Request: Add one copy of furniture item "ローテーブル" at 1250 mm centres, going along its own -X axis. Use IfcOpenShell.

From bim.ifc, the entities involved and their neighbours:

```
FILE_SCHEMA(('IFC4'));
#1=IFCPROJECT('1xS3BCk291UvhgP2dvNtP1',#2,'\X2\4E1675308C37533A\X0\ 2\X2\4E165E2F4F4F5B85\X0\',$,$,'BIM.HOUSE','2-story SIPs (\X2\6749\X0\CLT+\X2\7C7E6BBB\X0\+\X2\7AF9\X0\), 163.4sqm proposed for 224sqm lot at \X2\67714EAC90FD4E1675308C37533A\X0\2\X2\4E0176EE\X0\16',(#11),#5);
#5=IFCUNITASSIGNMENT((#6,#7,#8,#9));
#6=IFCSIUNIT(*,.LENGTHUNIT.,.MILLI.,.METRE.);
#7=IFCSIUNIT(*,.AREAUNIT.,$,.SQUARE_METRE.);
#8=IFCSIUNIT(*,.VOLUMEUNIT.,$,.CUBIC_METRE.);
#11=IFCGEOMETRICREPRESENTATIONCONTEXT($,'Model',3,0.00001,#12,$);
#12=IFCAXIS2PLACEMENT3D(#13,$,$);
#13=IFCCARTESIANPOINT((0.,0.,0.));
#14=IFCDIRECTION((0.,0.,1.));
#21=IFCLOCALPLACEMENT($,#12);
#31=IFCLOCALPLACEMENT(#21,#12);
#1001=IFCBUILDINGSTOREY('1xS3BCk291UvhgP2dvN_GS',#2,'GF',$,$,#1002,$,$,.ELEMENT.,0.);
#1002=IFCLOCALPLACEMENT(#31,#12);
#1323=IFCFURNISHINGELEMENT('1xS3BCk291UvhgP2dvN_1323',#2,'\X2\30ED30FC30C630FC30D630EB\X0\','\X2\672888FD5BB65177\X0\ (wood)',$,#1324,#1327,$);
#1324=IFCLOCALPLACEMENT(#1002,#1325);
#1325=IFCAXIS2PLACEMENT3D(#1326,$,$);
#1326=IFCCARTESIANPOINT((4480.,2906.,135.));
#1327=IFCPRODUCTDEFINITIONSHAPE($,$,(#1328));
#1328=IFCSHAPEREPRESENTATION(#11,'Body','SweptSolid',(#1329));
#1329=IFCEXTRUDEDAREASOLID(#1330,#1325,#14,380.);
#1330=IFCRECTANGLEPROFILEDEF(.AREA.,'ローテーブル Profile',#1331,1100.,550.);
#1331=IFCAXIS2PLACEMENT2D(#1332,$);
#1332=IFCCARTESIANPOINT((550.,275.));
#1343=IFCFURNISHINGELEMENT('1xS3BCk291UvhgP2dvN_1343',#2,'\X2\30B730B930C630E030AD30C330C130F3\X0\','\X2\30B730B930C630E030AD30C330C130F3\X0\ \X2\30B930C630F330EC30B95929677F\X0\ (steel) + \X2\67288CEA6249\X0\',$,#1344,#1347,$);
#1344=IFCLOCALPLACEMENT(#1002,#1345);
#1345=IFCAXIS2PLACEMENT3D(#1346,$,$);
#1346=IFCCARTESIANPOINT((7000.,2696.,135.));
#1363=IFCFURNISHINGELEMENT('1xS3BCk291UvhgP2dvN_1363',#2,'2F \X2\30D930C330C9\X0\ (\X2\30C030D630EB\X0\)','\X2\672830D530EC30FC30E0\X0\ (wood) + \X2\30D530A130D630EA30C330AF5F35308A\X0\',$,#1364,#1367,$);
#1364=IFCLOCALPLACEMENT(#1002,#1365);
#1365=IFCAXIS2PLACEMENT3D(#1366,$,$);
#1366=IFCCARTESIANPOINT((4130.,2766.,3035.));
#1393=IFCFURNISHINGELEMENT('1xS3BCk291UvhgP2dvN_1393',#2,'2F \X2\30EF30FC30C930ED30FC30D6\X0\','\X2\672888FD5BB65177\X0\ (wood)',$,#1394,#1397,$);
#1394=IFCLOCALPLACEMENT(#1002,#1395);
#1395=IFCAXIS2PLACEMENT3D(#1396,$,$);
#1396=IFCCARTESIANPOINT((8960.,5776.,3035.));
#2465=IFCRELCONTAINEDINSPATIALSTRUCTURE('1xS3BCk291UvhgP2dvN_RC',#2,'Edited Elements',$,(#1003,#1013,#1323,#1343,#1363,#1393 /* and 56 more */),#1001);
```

```python
import ifcopenshell
import ifcopenshell.api.geometry
import ifcopenshell.api.root
import ifcopenshell.util.element
import ifcopenshell.util.placement

model = ifcopenshell.open("bim.ifc")


def reuse_history(source, copy):
    """copy_class also copies each property set's owner history, people and application; keep the originals."""
    for rel in copy.IsDefinedBy:
        if rel.is_a("IfcRelDefinesByProperties") and (history := rel.RelatingPropertyDefinition.OwnerHistory):
            rel.RelatingPropertyDefinition.OwnerHistory = source.OwnerHistory
            ifcopenshell.util.element.remove_deep2(model, history)


source = model.by_guid("1xS3BCk291UvhgP2dvN_1323")
base = ifcopenshell.util.placement.get_local_placement(source.ObjectPlacement)
step = -base[:3, 0] * 1250.0

for i in range(1, 2):
    copy = ifcopenshell.api.root.copy_class(model, product=source)
    copy.Representation = ifcopenshell.util.element.copy_deep(
        model, source.Representation, exclude=["IfcGeometricRepresentationContext", "IfcRepresentationMap"]
    )
    reuse_history(source, copy)
    matrix = base.copy()
    matrix[:3, 3] += i * step
    print("added at", matrix[:3, 3].round(3) + 0.0)
    ifcopenshell.api.geometry.edit_object_placement(model, product=copy, matrix=matrix, is_si=False)

model.write("bim_edited.ifc")
```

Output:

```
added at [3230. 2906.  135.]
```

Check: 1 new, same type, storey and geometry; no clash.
